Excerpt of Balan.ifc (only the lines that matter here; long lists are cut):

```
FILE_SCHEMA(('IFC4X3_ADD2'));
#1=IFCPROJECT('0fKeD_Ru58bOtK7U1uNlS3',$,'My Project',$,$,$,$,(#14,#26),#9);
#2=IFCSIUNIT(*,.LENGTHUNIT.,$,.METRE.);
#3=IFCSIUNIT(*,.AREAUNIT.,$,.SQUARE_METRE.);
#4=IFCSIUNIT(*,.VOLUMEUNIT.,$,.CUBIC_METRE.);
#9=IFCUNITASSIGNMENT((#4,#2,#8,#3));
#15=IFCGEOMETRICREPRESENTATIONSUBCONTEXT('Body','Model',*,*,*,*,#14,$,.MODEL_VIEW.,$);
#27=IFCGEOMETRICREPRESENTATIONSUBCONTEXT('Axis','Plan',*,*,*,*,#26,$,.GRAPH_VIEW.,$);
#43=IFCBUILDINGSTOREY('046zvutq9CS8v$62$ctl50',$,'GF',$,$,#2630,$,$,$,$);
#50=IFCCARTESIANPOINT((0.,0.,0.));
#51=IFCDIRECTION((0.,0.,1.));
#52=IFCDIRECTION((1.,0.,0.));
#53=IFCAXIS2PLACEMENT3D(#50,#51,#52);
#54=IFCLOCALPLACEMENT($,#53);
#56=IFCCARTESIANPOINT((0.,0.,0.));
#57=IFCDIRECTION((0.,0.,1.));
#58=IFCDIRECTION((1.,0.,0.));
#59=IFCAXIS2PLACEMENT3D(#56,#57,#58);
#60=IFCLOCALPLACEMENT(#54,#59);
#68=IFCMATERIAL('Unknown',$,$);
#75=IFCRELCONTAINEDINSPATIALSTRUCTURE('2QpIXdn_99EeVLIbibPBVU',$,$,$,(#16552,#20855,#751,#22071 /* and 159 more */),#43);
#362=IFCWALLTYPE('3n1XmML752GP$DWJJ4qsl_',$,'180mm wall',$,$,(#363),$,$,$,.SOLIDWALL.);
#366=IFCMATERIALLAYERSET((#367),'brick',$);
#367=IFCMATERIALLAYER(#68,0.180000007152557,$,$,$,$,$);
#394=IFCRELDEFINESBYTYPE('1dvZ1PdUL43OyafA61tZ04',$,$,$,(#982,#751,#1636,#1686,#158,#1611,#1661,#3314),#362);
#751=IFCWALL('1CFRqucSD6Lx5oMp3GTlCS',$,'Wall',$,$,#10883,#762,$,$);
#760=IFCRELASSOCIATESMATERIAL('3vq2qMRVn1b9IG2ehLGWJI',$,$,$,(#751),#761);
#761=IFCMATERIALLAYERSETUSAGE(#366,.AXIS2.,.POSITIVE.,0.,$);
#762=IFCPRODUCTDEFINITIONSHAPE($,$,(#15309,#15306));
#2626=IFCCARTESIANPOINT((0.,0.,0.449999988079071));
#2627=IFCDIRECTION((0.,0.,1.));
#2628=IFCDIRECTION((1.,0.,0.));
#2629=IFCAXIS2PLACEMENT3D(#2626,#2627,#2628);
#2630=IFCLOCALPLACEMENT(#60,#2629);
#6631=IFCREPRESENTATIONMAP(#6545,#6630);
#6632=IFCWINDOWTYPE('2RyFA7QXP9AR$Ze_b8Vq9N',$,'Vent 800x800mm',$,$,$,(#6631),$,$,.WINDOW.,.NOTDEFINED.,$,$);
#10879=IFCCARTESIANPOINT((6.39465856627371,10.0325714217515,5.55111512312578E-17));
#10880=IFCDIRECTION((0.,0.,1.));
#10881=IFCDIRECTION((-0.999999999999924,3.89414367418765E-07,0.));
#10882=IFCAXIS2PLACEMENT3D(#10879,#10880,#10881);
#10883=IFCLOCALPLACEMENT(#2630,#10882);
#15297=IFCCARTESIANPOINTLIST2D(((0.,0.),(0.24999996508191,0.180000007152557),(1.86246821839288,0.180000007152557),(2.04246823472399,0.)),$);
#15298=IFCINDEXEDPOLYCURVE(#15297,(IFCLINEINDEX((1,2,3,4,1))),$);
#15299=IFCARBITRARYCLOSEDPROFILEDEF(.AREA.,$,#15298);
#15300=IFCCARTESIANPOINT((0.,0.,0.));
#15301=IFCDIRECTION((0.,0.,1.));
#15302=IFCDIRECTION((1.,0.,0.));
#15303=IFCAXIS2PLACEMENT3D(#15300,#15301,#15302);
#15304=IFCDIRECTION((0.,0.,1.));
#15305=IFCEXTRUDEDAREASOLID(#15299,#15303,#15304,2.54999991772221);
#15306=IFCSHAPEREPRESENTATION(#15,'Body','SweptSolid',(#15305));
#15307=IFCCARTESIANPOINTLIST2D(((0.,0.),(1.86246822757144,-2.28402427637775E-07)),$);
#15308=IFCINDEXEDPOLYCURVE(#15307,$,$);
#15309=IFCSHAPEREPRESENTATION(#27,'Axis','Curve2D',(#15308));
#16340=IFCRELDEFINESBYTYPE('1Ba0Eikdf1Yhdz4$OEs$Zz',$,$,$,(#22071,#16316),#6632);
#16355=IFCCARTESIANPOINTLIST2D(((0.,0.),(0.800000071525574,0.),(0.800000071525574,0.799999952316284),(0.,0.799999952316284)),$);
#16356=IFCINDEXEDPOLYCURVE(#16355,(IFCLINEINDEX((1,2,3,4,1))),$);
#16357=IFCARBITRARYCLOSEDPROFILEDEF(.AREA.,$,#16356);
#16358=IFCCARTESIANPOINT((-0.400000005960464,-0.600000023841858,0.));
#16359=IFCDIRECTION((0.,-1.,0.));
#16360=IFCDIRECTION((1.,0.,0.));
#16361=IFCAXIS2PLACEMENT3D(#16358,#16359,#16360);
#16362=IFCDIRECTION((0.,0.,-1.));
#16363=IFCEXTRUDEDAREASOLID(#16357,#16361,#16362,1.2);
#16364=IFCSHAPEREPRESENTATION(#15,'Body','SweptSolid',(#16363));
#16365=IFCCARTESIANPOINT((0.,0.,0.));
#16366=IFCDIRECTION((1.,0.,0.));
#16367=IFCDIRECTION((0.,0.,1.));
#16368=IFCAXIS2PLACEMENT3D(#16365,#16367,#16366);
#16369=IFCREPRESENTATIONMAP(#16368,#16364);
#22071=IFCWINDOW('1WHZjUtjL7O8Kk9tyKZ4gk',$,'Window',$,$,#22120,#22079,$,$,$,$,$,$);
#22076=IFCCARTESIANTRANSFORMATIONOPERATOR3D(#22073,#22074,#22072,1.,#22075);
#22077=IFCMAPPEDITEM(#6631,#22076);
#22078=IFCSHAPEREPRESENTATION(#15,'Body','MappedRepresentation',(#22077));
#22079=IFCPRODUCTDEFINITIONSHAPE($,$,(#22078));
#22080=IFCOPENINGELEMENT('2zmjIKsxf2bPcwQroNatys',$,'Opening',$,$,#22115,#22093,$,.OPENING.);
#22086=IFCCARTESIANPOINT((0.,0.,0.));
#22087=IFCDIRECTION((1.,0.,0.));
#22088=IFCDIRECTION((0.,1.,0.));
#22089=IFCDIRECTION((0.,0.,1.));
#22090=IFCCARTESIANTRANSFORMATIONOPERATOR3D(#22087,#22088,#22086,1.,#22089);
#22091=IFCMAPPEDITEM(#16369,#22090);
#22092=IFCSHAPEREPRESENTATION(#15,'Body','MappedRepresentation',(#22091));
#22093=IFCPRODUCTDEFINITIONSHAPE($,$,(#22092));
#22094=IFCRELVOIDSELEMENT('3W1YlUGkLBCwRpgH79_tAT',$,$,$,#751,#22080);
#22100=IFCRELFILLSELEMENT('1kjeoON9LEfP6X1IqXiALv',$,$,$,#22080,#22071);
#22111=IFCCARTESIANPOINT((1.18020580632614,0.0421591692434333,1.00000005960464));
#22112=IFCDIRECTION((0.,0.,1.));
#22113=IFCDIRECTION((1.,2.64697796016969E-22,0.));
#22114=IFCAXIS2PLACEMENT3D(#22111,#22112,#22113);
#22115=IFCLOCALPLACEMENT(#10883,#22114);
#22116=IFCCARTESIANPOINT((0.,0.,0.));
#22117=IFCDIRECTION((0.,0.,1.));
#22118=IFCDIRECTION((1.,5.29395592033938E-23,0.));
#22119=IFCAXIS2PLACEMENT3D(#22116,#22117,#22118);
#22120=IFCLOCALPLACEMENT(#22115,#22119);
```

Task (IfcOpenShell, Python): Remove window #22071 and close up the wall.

```python
import ifcopenshell
import ifcopenshell.api.feature
import ifcopenshell.api.root
import ifcopenshell.geom
import ifcopenshell.util.shape

model = ifcopenshell.open("Balan.ifc")
settings = ifcopenshell.geom.settings()


def volume(element):
    """Net volume in cubic metres, openings subtracted."""
    shape = ifcopenshell.geom.create_shape(settings, element)
    return ifcopenshell.util.shape.get_volume(shape.geometry)


window = model.by_guid("1WHZjUtjL7O8Kk9tyKZ4gk")
opening = window.FillsVoids[0].RelatingOpeningElement
wall = opening.VoidsElements[0].RelatingBuildingElement
before = volume(wall)

ifcopenshell.api.root.remove_product(model, product=window)
ifcopenshell.api.feature.remove_feature(model, feature=opening)

after = volume(wall)

print(f"wall volume {before:.3f} -> {after:.3f} m3")

model.write("Balan_updated.ifc")
```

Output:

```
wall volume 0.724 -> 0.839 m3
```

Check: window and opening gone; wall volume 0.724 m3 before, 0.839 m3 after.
